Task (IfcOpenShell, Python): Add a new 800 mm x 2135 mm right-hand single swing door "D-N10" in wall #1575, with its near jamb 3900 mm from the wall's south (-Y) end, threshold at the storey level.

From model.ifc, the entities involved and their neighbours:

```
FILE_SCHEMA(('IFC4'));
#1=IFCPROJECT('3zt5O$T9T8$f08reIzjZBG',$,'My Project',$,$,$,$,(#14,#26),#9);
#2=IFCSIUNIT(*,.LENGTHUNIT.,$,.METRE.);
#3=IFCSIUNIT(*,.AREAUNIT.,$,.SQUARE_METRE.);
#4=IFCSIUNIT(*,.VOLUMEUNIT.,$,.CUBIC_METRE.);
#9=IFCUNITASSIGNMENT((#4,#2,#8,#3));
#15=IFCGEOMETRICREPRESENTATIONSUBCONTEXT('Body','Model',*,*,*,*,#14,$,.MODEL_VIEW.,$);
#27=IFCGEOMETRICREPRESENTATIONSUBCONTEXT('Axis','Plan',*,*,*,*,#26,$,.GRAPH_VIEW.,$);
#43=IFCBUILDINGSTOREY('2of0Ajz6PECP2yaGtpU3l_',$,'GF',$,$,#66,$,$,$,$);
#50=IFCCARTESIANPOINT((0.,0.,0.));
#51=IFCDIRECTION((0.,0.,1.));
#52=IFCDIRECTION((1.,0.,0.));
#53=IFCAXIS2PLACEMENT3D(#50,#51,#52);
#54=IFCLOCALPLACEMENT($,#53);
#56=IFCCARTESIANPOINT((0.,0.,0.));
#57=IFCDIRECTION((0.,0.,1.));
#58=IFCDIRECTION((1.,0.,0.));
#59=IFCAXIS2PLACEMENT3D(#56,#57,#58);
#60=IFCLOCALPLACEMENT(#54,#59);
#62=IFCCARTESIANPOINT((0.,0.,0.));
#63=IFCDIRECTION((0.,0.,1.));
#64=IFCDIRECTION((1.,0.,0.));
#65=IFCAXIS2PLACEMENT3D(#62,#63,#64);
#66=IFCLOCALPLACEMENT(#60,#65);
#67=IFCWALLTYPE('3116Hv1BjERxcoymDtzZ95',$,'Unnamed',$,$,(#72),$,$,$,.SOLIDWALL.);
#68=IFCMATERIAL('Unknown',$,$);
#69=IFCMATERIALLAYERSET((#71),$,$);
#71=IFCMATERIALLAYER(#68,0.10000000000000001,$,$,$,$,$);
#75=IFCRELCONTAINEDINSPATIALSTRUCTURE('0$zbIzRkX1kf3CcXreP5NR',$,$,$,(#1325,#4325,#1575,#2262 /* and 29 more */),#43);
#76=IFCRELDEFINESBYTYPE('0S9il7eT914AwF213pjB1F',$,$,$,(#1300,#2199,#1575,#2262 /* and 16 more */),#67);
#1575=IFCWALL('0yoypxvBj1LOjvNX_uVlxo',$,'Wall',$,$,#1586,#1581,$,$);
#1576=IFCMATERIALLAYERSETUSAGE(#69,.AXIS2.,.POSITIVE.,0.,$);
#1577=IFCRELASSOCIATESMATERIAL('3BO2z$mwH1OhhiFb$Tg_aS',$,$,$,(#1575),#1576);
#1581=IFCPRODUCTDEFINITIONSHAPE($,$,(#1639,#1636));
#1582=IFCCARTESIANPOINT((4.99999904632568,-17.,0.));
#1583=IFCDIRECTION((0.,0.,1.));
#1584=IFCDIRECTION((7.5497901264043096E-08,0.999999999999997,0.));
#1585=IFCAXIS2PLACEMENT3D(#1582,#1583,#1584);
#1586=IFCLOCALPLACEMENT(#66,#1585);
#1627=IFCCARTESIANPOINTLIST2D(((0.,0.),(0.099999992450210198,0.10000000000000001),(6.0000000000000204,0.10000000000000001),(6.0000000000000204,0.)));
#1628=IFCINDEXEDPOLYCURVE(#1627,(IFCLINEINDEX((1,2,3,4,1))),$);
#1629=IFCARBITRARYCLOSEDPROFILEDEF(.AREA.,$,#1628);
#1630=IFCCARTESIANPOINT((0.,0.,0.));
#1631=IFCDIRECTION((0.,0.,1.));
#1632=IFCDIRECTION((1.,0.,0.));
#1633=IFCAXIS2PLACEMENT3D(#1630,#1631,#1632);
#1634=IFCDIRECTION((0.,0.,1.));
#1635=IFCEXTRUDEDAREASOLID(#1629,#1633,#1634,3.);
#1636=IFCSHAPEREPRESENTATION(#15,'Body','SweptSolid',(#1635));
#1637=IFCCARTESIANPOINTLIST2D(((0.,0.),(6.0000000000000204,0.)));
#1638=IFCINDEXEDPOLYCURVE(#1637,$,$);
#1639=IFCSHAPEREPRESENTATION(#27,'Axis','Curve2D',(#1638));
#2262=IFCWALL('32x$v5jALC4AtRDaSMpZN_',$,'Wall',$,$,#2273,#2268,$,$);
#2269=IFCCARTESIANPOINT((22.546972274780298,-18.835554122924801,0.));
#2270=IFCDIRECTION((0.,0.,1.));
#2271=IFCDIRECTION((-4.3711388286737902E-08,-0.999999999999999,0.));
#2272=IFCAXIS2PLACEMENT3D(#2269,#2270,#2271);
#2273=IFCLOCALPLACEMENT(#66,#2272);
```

```python
import numpy as np
import ifcopenshell
import ifcopenshell.api.feature
import ifcopenshell.api.geometry
import ifcopenshell.api.root
import ifcopenshell.api.spatial
import ifcopenshell.geom
import ifcopenshell.util.element
import ifcopenshell.util.placement
import ifcopenshell.util.representation
import ifcopenshell.util.shape
import ifcopenshell.util.unit

model = ifcopenshell.open("model.ifc")
unit_scale = ifcopenshell.util.unit.calculate_unit_scale(model)
settings = ifcopenshell.geom.settings()


def volume(element):
    """Net volume in cubic metres, openings subtracted."""
    shape = ifcopenshell.geom.create_shape(settings, element)
    return ifcopenshell.util.shape.get_volume(shape.geometry)


wall = model.by_id(1575)
storey = ifcopenshell.util.element.get_container(wall, ifc_class="IfcBuildingStorey")
context = ifcopenshell.util.representation.get_context(model, "Model", "Body", "MODEL_VIEW")
before = volume(wall)

width, height, from_end, sill = 0.8, 2.135, 3.9, 0.0  # metres

# The wall runs along its own X axis, and the end named is its -X end.
wall_shape = ifcopenshell.geom.create_shape(settings, wall)
x, y, z = ifcopenshell.util.shape.get_vertices(wall_shape.geometry).T
start = x.min() + from_end
face, thickness = float(y.min()), float(y.max() - y.min())
wall_matrix = ifcopenshell.util.placement.get_local_placement(wall.ObjectPlacement)
level = ifcopenshell.util.placement.get_local_placement(storey.ObjectPlacement)[2, 3]


def in_wall(x, y):
    """Placement at x, y metres in the wall's axes, at sill height."""
    matrix = wall_matrix.copy()
    matrix[:, 3] = wall_matrix @ np.array([x / unit_scale, y / unit_scale, 0.0, 1.0])
    matrix[2, 3] = level + sill / unit_scale
    return matrix


# Opening: a box that overshoots both wall faces by 50 mm.
opening = ifcopenshell.api.root.create_entity(model, ifc_class="IfcOpeningElement", predefined_type="OPENING")
box = ifcopenshell.api.geometry.add_wall_representation(
    model, context=context, length=width, height=height, thickness=thickness + 0.1
)
ifcopenshell.api.geometry.assign_representation(model, product=opening, representation=box)
ifcopenshell.api.geometry.edit_object_placement(model, product=opening, matrix=in_wall(start, face - 0.05), is_si=False)
ifcopenshell.api.feature.add_feature(model, feature=opening, element=wall)

door = ifcopenshell.api.root.create_entity(model, ifc_class="IfcDoor", name="D-N10", predefined_type="DOOR")
door.OverallWidth, door.OverallHeight = width / unit_scale, height / unit_scale
door.OperationType = "SINGLE_SWING_RIGHT"
body = ifcopenshell.api.geometry.add_door_representation(
    model,
    context=context,
    overall_width=door.OverallWidth,
    overall_height=door.OverallHeight,
    operation_type="SINGLE_SWING_RIGHT",
    lining_properties={"LiningDepth": thickness / unit_scale, "ThresholdDepth": thickness / unit_scale},
)
ifcopenshell.api.geometry.assign_representation(model, product=door, representation=body)
ifcopenshell.api.spatial.assign_container(model, products=[door], relating_structure=storey)
ifcopenshell.api.feature.add_filling(model, opening=opening, element=door)

# The lining spans the wall, so the door starts at the wall face.
ifcopenshell.api.geometry.edit_object_placement(model, product=door, matrix=in_wall(start, face), is_si=False)

after = volume(wall)

print(f"wall volume {before:.3f} -> {after:.3f} m3")

model.write("model_updated.ifc")
```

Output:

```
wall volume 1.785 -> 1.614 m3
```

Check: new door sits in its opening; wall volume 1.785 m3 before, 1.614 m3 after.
